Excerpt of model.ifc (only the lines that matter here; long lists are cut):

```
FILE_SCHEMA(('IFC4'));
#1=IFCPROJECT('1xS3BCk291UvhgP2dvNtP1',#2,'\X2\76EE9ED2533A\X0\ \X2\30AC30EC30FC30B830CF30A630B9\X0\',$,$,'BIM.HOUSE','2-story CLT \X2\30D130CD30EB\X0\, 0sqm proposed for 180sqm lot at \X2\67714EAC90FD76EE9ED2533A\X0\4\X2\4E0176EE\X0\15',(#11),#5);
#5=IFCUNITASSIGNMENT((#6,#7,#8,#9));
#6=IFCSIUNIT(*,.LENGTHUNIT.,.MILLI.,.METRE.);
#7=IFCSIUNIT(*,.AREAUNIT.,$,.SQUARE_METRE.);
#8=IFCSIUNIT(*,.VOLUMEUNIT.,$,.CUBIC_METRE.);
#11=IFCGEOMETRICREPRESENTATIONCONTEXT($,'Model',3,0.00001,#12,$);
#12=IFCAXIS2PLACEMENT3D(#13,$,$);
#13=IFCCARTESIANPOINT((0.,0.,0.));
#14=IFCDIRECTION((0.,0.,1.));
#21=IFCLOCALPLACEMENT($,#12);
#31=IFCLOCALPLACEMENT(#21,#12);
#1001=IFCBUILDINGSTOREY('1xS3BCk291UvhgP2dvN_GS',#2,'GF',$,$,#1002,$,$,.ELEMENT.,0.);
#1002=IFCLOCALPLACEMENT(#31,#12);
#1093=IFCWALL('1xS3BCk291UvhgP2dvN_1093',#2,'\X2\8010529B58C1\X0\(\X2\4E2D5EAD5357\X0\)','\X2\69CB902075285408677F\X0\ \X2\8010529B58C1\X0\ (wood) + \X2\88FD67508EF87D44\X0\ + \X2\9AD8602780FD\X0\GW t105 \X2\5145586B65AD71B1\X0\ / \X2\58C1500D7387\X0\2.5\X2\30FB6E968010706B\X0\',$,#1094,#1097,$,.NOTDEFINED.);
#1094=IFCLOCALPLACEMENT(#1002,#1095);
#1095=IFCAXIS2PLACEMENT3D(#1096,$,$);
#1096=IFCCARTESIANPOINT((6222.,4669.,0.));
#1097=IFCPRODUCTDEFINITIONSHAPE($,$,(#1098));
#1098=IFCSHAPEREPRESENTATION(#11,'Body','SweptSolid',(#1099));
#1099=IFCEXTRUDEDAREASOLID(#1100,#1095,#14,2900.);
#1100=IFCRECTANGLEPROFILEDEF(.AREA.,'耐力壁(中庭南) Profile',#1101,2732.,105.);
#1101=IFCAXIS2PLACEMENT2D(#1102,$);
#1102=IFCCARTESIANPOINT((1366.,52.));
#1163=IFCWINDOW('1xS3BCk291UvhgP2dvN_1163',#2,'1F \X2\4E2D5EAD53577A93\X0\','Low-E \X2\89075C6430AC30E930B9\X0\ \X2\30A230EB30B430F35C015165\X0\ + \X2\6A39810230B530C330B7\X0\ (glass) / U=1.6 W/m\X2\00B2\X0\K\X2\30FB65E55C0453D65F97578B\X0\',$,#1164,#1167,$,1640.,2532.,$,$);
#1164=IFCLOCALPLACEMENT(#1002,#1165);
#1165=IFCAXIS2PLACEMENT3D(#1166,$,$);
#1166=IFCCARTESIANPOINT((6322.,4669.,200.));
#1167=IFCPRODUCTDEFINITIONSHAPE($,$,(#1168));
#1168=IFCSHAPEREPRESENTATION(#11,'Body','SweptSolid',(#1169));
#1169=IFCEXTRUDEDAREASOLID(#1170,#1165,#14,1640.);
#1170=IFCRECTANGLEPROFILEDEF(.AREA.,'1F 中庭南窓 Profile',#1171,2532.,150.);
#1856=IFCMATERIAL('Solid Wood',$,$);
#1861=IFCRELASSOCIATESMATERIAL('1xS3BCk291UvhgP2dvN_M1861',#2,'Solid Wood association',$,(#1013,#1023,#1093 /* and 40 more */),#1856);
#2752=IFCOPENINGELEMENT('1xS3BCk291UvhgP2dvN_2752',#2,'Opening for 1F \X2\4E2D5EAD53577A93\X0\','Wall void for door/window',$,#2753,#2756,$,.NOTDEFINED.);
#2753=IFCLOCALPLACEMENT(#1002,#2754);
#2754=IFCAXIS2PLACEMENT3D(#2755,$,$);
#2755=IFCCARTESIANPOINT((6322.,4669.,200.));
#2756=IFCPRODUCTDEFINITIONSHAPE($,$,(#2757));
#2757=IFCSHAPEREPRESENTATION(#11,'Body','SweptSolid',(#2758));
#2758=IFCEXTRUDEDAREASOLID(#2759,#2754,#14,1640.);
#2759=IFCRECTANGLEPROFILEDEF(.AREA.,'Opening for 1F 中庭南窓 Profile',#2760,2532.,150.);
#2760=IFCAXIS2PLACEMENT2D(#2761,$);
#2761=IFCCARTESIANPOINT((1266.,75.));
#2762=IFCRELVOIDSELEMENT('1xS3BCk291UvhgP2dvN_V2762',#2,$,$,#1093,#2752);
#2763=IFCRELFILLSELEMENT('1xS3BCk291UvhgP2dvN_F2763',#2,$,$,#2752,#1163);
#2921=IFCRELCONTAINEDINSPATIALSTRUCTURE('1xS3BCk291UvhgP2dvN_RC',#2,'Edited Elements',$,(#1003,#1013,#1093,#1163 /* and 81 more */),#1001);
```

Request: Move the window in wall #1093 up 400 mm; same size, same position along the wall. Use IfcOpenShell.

```python
import numpy as np
import ifcopenshell
import ifcopenshell.api.geometry
import ifcopenshell.util.placement
import ifcopenshell.util.unit

model = ifcopenshell.open("model.ifc")
unit_scale = ifcopenshell.util.unit.calculate_unit_scale(model)

window = model.by_guid("1xS3BCk291UvhgP2dvN_1163")
opening = window.FillsVoids[0].RelatingOpeningElement
dz = 400.0

shift = np.array([0.0, 0.0, dz])
# The window is not placed relative to its opening, so move both.
for product in (opening, window):
    matrix = ifcopenshell.util.placement.get_local_placement(product.ObjectPlacement)
    matrix[:3, 3] += shift
    ifcopenshell.api.geometry.edit_object_placement(model, product=product, matrix=matrix, is_si=False)

print(f"moved by {dz * unit_scale:+.3f} m")

model.write("model-out.ifc")
```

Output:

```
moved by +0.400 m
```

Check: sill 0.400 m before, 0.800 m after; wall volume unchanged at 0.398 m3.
